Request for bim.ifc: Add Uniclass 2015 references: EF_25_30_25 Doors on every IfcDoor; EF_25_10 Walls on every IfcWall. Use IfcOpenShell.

First a look at what the model holds.

```python
import ifcopenshell

model = ifcopenshell.open("bim.ifc")
print(model.schema)
print("classifications:", [c.Name for c in model.by_type("IfcClassification")])
for ifc_class in ("IfcDoor", "IfcRoof", "IfcStair", "IfcWall", "IfcWindow"):
    print(ifc_class, len(model.by_type(ifc_class)))
```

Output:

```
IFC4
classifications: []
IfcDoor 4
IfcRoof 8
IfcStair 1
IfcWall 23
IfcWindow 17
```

```python
import ifcopenshell
import ifcopenshell.api.classification

model = ifcopenshell.open("bim.ifc")

system = ifcopenshell.api.classification.add_classification(model, classification="Uniclass 2015")

codes = {
    "IfcDoor": ("EF_25_30_25", "Doors"),
    "IfcWall": ("EF_25_10", "Walls"),
}
for ifc_class, (code, name) in codes.items():
    products = model.by_type(ifc_class)
    ifcopenshell.api.classification.add_reference(
        model, products=products, classification=system, identification=code, name=name
    )
    print(code, len(products))

model.write("bim_edited.ifc")
```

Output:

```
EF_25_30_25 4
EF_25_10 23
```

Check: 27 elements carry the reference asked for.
